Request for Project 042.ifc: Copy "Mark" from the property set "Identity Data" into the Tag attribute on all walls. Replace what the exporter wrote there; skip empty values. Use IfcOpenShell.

First a look at what the model holds.

```python
import ifcopenshell
import ifcopenshell.util.element

model = ifcopenshell.open("Project 042.ifc")
print(model.schema)
walls = model.by_type("IfcWall")
print(len(walls), "walls")
for e in walls[:8]:
    source = ifcopenshell.util.element.get_pset(e, "Identity Data", "Mark")
    target = e.Tag
    print(e.id(), repr(source), repr(target), sep=" | ")
```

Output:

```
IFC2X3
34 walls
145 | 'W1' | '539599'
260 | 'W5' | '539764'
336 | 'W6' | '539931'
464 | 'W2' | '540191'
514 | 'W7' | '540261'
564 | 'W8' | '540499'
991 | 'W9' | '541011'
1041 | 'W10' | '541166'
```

```python
import ifcopenshell
import ifcopenshell.util.element

model = ifcopenshell.open("Project 042.ifc")

count = 0
for e in model.by_type("IfcWall"):
    value = ifcopenshell.util.element.get_pset(e, "Identity Data", "Mark")
    current = e.Tag
    if not value or not value.strip() or current == value:
        continue
    e.Tag = value
    count += 1

print(count, "walls updated")

model.write("Project 042_v2.ifc")
```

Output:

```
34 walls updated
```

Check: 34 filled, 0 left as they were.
